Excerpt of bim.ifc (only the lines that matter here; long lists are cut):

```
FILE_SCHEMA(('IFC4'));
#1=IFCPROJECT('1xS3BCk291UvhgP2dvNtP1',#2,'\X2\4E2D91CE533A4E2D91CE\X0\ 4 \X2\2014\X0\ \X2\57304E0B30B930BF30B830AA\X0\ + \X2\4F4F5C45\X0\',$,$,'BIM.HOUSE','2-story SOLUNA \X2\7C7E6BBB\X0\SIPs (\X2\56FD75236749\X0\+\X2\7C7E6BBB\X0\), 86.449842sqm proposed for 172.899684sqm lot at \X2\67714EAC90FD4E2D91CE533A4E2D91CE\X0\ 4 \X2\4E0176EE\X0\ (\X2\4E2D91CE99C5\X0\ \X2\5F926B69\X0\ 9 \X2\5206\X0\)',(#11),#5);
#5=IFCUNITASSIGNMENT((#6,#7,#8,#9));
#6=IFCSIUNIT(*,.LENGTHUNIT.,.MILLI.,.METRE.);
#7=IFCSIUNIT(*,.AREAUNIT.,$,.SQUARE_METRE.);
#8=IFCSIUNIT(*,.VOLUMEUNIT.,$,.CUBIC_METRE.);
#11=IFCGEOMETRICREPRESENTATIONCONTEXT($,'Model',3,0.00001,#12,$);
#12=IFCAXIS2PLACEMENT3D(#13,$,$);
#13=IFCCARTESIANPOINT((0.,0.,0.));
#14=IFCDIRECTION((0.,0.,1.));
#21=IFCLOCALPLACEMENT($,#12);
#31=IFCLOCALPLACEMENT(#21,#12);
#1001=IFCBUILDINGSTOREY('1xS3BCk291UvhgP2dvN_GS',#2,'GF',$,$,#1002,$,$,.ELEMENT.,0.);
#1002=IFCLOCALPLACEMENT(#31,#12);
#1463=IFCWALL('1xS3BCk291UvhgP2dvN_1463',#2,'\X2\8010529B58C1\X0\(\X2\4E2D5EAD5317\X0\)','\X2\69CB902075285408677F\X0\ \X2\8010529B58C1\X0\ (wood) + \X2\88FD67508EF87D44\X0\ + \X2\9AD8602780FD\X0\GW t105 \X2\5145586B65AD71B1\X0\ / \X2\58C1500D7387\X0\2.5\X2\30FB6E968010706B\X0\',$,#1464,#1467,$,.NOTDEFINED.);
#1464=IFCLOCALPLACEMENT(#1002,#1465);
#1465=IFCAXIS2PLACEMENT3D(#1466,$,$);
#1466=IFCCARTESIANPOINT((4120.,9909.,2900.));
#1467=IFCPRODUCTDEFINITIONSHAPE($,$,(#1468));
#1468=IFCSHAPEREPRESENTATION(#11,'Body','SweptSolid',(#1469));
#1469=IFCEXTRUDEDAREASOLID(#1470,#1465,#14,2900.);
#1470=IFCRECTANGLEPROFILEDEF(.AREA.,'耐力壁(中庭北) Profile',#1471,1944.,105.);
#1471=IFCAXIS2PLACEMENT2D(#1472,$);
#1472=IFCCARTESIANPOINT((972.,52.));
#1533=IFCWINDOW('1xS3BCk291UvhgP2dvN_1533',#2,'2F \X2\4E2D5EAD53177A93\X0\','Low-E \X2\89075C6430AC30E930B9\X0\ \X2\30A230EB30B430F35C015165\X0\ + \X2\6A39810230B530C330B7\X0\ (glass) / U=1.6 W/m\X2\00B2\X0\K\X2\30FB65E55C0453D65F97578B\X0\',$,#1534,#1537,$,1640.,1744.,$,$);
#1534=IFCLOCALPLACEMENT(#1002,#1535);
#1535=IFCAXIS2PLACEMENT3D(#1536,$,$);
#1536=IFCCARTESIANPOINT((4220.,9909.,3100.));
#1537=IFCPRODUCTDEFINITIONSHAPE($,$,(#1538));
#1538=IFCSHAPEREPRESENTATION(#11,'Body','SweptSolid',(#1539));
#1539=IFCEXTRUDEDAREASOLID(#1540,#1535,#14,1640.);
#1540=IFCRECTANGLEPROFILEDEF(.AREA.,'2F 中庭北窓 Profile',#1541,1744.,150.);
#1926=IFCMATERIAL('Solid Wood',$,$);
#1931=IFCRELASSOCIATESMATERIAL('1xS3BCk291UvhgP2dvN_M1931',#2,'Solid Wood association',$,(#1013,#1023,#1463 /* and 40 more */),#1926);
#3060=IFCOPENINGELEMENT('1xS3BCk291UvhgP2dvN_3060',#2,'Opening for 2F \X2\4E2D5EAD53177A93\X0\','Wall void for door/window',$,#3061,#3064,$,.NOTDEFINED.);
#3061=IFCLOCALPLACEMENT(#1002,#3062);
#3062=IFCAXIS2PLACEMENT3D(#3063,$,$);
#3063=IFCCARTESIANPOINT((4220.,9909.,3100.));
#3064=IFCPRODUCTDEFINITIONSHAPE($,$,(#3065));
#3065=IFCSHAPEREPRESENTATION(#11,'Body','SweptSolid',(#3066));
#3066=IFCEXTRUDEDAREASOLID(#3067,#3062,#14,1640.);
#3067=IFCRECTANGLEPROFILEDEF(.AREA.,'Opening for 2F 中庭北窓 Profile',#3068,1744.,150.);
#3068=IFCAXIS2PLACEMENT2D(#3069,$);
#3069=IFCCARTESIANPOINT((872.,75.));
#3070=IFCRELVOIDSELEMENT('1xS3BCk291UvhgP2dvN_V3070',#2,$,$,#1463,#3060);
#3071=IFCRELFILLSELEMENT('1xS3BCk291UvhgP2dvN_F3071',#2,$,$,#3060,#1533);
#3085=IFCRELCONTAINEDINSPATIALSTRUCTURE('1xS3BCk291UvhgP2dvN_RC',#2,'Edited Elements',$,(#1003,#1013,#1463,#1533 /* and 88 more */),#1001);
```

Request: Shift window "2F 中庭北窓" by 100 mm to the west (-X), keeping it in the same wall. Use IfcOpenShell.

```python
import ifcopenshell
import ifcopenshell.api.geometry
import ifcopenshell.util.placement

model = ifcopenshell.open("bim.ifc")

window = model.by_guid("1xS3BCk291UvhgP2dvN_1533")
opening = window.FillsVoids[0].RelatingOpeningElement
wall = opening.VoidsElements[0].RelatingBuildingElement

wall_matrix = ifcopenshell.util.placement.get_local_placement(wall.ObjectPlacement)
shift = wall_matrix[:3, 0] * -100.0
before = ifcopenshell.util.placement.get_local_placement(window.ObjectPlacement)[:3, 3].copy()

# The window is not placed relative to its opening, so move both.
for product in (opening, window):
    matrix = ifcopenshell.util.placement.get_local_placement(product.ObjectPlacement)
    matrix[:3, 3] += shift
    ifcopenshell.api.geometry.edit_object_placement(model, product=product, matrix=matrix, is_si=False)

after = ifcopenshell.util.placement.get_local_placement(window.ObjectPlacement)[:3, 3]
print("window moved by", (after - before).round(3) + 0.0)

model.write("bim_v2.ifc")
```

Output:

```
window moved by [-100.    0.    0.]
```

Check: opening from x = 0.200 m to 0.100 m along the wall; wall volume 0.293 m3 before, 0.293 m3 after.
